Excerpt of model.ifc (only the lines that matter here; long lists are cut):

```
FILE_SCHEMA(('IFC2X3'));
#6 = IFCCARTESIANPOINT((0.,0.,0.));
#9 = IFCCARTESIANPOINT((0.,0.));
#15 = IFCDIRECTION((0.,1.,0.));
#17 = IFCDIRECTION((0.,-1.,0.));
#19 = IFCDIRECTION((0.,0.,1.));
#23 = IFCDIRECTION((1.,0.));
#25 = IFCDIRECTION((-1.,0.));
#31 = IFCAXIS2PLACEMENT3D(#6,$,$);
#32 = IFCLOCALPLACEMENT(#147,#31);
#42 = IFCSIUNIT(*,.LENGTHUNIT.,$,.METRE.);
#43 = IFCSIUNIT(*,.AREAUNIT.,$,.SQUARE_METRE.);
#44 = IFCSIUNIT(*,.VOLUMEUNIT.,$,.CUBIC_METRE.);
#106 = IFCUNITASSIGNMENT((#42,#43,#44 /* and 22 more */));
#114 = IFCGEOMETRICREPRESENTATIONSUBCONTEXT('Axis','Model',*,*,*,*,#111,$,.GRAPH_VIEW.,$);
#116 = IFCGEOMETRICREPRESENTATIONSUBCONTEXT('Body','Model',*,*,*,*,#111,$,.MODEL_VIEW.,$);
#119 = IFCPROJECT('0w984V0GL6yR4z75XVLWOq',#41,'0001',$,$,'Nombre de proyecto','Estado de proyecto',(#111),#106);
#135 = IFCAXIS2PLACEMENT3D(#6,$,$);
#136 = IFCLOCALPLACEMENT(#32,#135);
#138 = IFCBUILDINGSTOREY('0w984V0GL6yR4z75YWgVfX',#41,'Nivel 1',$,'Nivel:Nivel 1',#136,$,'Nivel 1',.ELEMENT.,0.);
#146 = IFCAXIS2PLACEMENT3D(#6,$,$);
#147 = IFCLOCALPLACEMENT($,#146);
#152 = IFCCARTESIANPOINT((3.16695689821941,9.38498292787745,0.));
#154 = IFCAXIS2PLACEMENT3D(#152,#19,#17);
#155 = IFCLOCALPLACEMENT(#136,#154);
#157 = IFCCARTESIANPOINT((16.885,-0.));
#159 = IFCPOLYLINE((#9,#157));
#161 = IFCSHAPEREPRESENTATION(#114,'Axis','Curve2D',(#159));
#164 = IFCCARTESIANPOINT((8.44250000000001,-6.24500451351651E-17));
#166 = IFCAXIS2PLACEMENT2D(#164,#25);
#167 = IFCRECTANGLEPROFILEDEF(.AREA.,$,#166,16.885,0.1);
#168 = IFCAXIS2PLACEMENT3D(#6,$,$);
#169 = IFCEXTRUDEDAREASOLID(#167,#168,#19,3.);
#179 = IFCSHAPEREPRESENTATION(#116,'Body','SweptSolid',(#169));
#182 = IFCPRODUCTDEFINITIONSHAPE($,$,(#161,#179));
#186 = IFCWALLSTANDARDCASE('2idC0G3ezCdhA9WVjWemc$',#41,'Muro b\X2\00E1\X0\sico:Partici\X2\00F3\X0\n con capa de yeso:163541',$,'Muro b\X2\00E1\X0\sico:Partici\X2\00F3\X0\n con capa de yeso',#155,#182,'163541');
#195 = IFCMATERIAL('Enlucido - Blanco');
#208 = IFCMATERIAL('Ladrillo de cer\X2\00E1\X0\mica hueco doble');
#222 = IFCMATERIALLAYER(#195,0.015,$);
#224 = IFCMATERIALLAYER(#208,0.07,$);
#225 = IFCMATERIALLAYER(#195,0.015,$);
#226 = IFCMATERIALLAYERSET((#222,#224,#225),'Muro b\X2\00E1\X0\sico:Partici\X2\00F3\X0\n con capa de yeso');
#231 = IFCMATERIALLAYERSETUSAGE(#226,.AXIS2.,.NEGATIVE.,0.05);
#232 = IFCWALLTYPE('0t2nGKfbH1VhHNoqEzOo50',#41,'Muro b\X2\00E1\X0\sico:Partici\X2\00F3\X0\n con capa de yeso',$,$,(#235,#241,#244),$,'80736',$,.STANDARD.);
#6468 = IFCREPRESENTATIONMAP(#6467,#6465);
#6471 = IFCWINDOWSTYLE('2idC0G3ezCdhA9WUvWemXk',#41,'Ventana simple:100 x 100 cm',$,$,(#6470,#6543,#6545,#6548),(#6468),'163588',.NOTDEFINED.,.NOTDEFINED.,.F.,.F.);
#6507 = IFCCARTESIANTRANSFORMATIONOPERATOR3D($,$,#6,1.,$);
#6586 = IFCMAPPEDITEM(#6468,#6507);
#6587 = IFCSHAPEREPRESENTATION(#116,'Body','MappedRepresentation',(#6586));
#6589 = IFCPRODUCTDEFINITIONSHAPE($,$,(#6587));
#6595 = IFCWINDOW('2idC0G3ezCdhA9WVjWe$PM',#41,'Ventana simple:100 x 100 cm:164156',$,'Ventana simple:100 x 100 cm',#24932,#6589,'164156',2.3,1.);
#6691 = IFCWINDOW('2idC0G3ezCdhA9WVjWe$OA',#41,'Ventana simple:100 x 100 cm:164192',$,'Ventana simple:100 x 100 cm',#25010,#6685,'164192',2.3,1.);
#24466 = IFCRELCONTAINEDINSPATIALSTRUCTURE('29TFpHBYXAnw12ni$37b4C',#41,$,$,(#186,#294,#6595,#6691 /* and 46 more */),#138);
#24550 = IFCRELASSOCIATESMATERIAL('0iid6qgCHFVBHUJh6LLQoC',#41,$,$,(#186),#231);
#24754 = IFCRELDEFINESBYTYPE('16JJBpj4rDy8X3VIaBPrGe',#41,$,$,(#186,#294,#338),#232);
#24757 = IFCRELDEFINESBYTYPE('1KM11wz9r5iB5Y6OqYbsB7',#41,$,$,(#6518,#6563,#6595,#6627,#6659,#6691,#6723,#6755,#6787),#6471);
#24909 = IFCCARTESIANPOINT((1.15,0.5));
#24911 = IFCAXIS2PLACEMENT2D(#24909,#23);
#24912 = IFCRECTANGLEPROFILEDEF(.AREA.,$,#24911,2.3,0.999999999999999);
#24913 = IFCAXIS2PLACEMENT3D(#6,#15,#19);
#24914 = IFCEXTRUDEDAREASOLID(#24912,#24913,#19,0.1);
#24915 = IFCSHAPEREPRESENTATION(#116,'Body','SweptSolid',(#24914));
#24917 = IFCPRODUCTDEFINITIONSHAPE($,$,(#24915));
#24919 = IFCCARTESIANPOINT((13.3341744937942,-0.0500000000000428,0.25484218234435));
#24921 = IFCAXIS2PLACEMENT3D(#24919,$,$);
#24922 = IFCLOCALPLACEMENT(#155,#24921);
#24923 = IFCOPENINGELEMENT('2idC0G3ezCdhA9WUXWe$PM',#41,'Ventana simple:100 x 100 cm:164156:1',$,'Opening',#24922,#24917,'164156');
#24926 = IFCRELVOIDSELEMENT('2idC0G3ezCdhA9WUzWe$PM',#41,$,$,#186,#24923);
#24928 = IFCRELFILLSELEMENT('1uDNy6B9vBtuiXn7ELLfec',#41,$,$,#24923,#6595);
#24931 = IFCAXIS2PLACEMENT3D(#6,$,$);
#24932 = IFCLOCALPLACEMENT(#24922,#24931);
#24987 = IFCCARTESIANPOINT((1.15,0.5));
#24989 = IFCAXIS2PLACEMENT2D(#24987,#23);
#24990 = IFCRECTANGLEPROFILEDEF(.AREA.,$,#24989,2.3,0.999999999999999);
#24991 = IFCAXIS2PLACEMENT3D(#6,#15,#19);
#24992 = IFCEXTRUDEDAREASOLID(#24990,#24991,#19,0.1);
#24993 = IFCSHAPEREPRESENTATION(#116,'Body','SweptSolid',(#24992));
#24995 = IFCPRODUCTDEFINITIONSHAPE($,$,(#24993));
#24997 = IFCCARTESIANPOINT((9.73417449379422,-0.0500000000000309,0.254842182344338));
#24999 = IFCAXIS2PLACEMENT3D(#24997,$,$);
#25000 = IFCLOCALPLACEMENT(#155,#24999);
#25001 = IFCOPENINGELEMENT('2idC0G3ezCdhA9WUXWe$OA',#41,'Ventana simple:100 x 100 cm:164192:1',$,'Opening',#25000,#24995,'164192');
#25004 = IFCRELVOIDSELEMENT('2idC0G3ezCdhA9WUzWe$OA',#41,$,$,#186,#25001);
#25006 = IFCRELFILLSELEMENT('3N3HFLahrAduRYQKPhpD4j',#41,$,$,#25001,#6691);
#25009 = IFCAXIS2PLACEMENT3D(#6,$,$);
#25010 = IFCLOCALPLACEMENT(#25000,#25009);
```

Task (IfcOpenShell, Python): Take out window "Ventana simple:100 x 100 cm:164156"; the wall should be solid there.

```python
import ifcopenshell
import ifcopenshell.api.feature
import ifcopenshell.api.root
import ifcopenshell.geom
import ifcopenshell.util.shape

model = ifcopenshell.open("model.ifc")
settings = ifcopenshell.geom.settings()


def volume(element):
    """Net volume in cubic metres, openings subtracted."""
    shape = ifcopenshell.geom.create_shape(settings, element)
    return ifcopenshell.util.shape.get_volume(shape.geometry)


window = model.by_guid("2idC0G3ezCdhA9WVjWe$PM")
opening = window.FillsVoids[0].RelatingOpeningElement
wall = opening.VoidsElements[0].RelatingBuildingElement
before = volume(wall)

ifcopenshell.api.root.remove_product(model, product=window)
ifcopenshell.api.feature.remove_feature(model, feature=opening)

after = volume(wall)

print(f"wall volume {before:.3f} -> {after:.3f} m3")

model.write("model_edited.ifc")
```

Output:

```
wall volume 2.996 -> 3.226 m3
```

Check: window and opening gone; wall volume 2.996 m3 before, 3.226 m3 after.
